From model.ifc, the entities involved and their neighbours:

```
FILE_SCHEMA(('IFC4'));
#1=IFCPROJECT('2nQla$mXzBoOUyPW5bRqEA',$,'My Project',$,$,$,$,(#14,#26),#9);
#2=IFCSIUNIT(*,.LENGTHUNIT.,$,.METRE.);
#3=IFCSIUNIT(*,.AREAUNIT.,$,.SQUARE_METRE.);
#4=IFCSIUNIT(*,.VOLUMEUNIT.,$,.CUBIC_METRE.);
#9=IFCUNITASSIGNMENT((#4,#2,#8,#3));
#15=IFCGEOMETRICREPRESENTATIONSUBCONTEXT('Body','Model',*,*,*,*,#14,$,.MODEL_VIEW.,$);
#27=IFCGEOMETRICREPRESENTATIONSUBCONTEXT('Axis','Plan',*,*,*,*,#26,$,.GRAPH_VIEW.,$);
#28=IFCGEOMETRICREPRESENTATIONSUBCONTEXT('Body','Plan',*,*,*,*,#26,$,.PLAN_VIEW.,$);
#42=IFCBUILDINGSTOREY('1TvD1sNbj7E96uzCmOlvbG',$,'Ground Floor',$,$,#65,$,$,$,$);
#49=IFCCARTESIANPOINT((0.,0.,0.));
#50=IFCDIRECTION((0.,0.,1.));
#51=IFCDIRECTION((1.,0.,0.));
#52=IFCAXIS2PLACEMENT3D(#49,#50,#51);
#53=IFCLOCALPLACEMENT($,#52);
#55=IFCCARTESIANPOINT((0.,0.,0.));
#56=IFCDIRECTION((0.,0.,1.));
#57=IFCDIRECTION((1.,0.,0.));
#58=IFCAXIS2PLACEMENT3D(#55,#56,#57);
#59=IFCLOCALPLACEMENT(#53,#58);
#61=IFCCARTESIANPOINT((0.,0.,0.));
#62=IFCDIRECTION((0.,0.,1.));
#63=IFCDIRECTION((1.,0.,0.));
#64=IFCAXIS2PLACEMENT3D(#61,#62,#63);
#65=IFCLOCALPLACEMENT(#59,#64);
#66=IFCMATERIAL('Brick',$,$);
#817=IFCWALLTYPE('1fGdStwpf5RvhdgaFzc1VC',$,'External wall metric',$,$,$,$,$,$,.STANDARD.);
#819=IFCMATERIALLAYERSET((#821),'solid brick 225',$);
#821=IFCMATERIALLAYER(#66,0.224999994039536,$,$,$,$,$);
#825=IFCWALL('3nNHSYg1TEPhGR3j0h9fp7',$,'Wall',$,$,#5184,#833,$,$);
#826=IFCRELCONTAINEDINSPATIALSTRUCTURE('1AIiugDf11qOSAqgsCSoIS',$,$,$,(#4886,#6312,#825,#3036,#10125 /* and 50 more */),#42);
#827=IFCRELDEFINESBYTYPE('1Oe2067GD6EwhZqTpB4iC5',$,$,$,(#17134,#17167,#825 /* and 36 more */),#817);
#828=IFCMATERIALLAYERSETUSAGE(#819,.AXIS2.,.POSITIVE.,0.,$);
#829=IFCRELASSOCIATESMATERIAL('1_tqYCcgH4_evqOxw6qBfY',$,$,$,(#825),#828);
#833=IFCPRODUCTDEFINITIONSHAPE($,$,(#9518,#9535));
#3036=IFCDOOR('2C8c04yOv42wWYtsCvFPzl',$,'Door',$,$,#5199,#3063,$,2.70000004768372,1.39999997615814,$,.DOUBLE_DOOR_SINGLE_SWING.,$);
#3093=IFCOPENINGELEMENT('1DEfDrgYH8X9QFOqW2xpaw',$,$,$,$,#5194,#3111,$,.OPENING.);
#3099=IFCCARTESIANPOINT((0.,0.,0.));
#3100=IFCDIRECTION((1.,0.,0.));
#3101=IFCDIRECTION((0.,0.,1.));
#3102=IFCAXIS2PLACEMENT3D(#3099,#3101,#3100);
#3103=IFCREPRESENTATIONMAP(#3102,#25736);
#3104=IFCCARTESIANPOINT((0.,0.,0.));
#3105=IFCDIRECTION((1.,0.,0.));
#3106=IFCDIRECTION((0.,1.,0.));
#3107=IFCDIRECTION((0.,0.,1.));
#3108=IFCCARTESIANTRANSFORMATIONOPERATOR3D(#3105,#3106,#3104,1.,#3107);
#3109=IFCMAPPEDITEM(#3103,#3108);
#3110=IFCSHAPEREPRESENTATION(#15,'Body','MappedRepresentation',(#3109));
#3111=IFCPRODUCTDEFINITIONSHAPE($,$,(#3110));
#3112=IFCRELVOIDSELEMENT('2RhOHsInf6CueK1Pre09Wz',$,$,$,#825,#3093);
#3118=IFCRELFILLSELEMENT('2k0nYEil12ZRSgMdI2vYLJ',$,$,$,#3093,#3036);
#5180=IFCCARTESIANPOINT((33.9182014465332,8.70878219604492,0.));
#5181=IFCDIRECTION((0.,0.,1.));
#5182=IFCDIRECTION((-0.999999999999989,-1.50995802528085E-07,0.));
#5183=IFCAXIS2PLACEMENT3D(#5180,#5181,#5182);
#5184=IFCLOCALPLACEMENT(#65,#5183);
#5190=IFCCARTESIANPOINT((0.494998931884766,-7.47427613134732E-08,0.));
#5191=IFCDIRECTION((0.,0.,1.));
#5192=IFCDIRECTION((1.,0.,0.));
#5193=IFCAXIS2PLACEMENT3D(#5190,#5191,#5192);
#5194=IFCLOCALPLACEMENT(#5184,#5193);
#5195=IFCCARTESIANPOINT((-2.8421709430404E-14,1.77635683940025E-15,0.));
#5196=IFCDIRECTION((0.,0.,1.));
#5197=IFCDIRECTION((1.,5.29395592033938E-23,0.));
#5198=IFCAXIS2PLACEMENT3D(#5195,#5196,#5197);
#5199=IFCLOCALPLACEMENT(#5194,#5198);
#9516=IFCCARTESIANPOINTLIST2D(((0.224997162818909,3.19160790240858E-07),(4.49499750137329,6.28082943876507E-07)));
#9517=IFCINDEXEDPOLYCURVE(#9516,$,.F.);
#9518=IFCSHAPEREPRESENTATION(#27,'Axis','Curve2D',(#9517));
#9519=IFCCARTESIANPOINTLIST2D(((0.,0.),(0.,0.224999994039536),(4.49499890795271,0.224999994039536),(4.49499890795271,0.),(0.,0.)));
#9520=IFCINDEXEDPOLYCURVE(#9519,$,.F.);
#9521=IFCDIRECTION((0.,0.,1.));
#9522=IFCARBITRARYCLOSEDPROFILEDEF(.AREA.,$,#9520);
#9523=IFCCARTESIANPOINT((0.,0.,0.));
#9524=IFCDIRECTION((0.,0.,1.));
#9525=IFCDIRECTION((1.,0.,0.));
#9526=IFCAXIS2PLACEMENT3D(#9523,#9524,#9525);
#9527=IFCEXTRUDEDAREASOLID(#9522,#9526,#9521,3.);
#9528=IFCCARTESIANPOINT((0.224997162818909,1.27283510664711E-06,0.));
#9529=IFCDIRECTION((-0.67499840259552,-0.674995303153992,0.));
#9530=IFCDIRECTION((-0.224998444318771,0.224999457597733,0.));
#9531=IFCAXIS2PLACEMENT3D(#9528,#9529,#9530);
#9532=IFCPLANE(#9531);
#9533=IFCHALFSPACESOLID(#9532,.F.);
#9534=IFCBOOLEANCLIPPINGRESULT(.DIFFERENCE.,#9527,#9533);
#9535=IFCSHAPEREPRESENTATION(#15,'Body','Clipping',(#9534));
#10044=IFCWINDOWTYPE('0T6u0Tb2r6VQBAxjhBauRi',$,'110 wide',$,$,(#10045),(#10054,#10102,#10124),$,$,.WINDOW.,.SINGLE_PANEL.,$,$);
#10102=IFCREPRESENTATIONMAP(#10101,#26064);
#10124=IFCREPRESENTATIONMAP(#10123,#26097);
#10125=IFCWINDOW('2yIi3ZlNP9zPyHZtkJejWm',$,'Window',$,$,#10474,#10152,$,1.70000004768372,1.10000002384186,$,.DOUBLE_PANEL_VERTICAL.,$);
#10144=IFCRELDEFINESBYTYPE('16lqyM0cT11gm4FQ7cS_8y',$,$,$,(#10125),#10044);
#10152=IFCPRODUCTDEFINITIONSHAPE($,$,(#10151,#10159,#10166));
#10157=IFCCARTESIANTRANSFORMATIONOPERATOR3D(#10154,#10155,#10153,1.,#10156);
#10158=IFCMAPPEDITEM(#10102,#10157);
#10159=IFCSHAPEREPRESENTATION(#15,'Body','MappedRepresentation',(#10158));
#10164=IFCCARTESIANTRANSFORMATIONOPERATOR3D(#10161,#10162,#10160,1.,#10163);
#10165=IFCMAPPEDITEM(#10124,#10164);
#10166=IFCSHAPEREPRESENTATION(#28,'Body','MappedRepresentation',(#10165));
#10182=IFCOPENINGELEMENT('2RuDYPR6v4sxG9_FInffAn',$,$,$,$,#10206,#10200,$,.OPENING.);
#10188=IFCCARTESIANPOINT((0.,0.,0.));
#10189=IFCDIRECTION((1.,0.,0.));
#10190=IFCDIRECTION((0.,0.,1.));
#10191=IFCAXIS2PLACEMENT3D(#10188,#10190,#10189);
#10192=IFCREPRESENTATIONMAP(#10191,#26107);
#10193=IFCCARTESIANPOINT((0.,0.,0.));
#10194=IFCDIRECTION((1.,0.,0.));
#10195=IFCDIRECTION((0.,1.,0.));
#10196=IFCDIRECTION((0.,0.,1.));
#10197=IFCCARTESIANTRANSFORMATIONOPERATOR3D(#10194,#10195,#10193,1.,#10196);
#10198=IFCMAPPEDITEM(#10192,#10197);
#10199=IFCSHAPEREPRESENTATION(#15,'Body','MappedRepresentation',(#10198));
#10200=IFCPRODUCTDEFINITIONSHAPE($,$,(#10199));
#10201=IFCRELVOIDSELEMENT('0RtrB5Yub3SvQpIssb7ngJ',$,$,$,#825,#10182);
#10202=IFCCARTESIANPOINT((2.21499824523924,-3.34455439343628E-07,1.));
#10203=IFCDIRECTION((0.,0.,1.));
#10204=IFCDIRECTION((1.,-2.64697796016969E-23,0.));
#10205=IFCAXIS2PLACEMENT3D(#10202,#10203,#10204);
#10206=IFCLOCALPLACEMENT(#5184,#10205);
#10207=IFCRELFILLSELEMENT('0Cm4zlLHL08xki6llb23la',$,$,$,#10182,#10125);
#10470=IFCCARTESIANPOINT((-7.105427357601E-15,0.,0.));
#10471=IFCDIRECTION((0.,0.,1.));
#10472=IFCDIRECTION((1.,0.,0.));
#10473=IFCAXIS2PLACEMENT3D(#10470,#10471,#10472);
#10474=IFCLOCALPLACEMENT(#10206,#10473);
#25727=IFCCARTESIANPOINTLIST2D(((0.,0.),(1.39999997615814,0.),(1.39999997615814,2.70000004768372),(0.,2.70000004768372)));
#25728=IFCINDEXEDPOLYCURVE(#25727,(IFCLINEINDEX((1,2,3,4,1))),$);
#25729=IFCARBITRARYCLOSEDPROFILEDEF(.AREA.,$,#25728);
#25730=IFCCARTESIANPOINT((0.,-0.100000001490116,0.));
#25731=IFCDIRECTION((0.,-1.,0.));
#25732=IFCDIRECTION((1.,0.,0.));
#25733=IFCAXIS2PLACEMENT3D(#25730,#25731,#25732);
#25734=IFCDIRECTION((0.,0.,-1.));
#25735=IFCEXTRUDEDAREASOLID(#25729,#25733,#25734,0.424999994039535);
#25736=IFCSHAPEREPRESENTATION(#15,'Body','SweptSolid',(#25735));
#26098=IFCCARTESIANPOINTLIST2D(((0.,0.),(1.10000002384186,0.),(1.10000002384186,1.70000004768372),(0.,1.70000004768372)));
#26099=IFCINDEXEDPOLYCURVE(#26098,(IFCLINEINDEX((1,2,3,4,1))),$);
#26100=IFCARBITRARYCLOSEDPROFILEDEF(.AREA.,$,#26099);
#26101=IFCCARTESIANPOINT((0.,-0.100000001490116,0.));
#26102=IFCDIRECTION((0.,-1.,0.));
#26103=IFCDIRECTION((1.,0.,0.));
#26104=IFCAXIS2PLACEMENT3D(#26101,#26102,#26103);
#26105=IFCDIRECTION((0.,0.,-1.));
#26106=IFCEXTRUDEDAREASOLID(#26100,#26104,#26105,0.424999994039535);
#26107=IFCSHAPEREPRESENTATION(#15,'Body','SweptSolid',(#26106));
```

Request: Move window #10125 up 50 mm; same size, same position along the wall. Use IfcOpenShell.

```python
import numpy as np
import ifcopenshell
import ifcopenshell.api.geometry
import ifcopenshell.util.placement
import ifcopenshell.util.unit

model = ifcopenshell.open("model.ifc")
unit_scale = ifcopenshell.util.unit.calculate_unit_scale(model)

window = model.by_guid("2yIi3ZlNP9zPyHZtkJejWm")
opening = window.FillsVoids[0].RelatingOpeningElement
dz = 0.05

shift = np.array([0.0, 0.0, dz])
# The window is placed relative to its opening, so it follows when the opening moves.
matrix = ifcopenshell.util.placement.get_local_placement(opening.ObjectPlacement)
matrix[:3, 3] += shift
ifcopenshell.api.geometry.edit_object_placement(
    model, product=opening, matrix=matrix, is_si=False, should_transform_children=True
)

print(f"moved by {dz * unit_scale:+.3f} m")

model.write("model_updated.ifc")
```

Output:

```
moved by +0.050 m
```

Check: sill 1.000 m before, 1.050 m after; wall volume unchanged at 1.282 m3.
